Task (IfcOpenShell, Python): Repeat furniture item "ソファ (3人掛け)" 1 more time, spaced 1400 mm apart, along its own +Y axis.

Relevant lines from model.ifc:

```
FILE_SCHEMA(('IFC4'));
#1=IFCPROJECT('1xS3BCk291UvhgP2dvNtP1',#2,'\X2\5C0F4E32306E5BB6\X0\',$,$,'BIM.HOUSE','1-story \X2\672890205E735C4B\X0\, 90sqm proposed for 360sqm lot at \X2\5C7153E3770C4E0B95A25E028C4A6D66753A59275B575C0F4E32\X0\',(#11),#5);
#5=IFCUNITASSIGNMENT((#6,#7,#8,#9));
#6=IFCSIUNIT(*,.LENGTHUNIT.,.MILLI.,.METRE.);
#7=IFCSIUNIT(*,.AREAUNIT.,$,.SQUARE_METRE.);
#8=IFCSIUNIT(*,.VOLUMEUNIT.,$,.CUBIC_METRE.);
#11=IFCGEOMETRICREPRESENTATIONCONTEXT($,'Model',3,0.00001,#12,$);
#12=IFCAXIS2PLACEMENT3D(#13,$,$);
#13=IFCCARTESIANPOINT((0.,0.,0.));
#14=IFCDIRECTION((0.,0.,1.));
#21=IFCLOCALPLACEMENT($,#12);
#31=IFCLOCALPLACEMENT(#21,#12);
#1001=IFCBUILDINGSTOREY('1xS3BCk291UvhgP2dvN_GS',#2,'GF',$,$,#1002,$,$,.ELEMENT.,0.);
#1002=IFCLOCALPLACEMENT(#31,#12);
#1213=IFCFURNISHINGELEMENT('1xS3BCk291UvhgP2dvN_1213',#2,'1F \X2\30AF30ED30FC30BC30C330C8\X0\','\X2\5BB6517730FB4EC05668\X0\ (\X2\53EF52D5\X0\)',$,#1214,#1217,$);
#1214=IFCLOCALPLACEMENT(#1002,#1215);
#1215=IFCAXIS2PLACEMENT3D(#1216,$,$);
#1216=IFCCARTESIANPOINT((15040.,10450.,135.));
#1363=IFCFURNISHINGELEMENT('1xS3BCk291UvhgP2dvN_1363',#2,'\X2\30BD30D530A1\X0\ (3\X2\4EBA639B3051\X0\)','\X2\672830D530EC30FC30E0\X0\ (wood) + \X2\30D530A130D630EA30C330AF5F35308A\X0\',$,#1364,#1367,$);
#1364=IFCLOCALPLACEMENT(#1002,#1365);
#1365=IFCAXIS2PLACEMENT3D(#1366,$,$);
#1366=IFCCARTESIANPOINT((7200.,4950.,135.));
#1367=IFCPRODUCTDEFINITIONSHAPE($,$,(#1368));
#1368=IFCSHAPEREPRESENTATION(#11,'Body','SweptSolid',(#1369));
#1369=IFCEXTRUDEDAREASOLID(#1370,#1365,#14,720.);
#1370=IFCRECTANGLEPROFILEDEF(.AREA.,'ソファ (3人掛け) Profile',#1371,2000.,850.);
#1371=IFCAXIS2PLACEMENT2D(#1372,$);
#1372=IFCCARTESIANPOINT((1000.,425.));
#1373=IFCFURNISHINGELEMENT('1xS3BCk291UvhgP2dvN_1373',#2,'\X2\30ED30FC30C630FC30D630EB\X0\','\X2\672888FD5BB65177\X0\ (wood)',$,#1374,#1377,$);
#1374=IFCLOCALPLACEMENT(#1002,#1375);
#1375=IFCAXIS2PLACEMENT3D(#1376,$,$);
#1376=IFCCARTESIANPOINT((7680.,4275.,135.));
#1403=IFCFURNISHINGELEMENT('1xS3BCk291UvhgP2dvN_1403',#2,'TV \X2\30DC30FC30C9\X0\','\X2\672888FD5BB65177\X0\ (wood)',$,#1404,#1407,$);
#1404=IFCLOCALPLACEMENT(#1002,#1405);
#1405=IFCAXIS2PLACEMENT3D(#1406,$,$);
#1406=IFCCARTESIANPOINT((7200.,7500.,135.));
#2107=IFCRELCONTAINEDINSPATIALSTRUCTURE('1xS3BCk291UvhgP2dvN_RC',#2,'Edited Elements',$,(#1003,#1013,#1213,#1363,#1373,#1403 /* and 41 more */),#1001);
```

```python
import ifcopenshell
import ifcopenshell.api.geometry
import ifcopenshell.api.root
import ifcopenshell.util.element
import ifcopenshell.util.placement
import ifcopenshell.util.unit

model = ifcopenshell.open("model.ifc")
unit_scale = ifcopenshell.util.unit.calculate_unit_scale(model)


def reuse_history(source, copy):
    """copy_class also copies each property set's owner history, people and application; keep the originals."""
    for rel in copy.IsDefinedBy:
        if rel.is_a("IfcRelDefinesByProperties") and (history := rel.RelatingPropertyDefinition.OwnerHistory):
            rel.RelatingPropertyDefinition.OwnerHistory = source.OwnerHistory
            ifcopenshell.util.element.remove_deep2(model, history)


source = model.by_id(1363)
base = ifcopenshell.util.placement.get_local_placement(source.ObjectPlacement)
step = base[:3, 1] * 1.4 / unit_scale

for i in range(1, 2):
    copy = ifcopenshell.api.root.copy_class(model, product=source)
    copy.Representation = ifcopenshell.util.element.copy_deep(
        model, source.Representation, exclude=["IfcGeometricRepresentationContext", "IfcRepresentationMap"]
    )
    reuse_history(source, copy)
    matrix = base.copy()
    matrix[:3, 3] += i * step
    print("added at", matrix[:3, 3].round(3) + 0.0)
    ifcopenshell.api.geometry.edit_object_placement(model, product=copy, matrix=matrix, is_si=False)

model.write("model_v2.ifc")
```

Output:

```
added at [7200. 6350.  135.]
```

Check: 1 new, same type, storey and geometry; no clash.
